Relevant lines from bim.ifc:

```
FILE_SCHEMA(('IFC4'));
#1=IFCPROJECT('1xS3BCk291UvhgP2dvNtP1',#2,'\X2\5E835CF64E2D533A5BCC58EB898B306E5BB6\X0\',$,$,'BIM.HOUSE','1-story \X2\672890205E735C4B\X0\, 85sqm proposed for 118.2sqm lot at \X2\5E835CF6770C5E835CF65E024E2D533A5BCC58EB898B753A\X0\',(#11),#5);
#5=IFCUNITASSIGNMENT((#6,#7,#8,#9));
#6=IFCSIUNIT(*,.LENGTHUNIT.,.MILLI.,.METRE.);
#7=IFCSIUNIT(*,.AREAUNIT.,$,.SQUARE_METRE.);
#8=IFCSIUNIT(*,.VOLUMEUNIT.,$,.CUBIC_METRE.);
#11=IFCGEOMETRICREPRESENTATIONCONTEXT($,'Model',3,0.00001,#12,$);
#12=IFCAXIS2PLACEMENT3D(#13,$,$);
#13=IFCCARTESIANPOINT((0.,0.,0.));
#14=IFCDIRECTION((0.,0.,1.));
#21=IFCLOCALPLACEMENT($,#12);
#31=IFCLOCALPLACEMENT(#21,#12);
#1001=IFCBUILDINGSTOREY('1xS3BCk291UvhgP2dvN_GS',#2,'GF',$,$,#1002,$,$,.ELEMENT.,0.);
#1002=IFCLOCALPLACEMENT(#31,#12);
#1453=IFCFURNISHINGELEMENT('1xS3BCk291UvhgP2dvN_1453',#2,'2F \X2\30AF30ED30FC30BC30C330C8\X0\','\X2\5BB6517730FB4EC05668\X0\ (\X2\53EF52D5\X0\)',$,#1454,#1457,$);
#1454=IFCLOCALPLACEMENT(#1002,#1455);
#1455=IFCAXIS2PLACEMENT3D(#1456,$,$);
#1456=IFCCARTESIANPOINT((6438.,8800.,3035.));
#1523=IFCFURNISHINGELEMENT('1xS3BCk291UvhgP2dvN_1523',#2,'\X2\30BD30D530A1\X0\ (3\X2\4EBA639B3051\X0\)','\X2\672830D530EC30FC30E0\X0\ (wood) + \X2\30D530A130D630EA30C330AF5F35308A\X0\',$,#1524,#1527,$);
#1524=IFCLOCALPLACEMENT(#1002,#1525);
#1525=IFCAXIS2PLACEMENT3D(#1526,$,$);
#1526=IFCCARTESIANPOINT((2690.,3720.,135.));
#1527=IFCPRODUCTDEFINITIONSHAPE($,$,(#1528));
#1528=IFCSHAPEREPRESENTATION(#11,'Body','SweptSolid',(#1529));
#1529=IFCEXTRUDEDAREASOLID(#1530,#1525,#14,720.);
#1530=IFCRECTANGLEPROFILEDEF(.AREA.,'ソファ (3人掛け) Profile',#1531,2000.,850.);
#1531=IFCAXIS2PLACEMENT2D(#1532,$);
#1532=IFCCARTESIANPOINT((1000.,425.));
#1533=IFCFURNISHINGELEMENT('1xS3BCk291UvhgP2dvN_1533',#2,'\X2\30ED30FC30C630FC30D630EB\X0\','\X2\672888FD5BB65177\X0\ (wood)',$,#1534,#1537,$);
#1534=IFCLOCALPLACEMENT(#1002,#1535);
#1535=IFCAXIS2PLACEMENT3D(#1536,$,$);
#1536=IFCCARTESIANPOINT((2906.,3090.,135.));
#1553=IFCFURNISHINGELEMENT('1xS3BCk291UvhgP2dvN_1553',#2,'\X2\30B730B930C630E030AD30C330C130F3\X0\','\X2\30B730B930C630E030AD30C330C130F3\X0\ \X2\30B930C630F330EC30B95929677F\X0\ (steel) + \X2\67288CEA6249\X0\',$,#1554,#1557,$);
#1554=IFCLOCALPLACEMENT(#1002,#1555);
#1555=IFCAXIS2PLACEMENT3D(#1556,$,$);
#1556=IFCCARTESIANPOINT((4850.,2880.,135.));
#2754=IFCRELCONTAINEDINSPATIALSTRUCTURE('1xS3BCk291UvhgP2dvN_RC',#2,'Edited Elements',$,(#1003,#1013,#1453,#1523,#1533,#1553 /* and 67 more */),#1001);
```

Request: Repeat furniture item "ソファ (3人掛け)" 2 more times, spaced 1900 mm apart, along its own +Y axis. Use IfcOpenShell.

```python
import ifcopenshell
import ifcopenshell.api.geometry
import ifcopenshell.api.root
import ifcopenshell.util.element
import ifcopenshell.util.placement
import ifcopenshell.util.unit

model = ifcopenshell.open("bim.ifc")
unit_scale = ifcopenshell.util.unit.calculate_unit_scale(model)


def reuse_history(source, copy):
    """copy_class also copies each property set's owner history, people and application; keep the originals."""
    for rel in copy.IsDefinedBy:
        if rel.is_a("IfcRelDefinesByProperties") and (history := rel.RelatingPropertyDefinition.OwnerHistory):
            rel.RelatingPropertyDefinition.OwnerHistory = source.OwnerHistory
            ifcopenshell.util.element.remove_deep2(model, history)


source = model.by_guid("1xS3BCk291UvhgP2dvN_1523")
base = ifcopenshell.util.placement.get_local_placement(source.ObjectPlacement)
step = base[:3, 1] * 1.9 / unit_scale

for i in range(1, 3):
    copy = ifcopenshell.api.root.copy_class(model, product=source)
    copy.Representation = ifcopenshell.util.element.copy_deep(
        model, source.Representation, exclude=["IfcGeometricRepresentationContext", "IfcRepresentationMap"]
    )
    reuse_history(source, copy)
    matrix = base.copy()
    matrix[:3, 3] += i * step
    print("added at", matrix[:3, 3].round(3) + 0.0)
    ifcopenshell.api.geometry.edit_object_placement(model, product=copy, matrix=matrix, is_si=False)

model.write("bim_rev.ifc")
```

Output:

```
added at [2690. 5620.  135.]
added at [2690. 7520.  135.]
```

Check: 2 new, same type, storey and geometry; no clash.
